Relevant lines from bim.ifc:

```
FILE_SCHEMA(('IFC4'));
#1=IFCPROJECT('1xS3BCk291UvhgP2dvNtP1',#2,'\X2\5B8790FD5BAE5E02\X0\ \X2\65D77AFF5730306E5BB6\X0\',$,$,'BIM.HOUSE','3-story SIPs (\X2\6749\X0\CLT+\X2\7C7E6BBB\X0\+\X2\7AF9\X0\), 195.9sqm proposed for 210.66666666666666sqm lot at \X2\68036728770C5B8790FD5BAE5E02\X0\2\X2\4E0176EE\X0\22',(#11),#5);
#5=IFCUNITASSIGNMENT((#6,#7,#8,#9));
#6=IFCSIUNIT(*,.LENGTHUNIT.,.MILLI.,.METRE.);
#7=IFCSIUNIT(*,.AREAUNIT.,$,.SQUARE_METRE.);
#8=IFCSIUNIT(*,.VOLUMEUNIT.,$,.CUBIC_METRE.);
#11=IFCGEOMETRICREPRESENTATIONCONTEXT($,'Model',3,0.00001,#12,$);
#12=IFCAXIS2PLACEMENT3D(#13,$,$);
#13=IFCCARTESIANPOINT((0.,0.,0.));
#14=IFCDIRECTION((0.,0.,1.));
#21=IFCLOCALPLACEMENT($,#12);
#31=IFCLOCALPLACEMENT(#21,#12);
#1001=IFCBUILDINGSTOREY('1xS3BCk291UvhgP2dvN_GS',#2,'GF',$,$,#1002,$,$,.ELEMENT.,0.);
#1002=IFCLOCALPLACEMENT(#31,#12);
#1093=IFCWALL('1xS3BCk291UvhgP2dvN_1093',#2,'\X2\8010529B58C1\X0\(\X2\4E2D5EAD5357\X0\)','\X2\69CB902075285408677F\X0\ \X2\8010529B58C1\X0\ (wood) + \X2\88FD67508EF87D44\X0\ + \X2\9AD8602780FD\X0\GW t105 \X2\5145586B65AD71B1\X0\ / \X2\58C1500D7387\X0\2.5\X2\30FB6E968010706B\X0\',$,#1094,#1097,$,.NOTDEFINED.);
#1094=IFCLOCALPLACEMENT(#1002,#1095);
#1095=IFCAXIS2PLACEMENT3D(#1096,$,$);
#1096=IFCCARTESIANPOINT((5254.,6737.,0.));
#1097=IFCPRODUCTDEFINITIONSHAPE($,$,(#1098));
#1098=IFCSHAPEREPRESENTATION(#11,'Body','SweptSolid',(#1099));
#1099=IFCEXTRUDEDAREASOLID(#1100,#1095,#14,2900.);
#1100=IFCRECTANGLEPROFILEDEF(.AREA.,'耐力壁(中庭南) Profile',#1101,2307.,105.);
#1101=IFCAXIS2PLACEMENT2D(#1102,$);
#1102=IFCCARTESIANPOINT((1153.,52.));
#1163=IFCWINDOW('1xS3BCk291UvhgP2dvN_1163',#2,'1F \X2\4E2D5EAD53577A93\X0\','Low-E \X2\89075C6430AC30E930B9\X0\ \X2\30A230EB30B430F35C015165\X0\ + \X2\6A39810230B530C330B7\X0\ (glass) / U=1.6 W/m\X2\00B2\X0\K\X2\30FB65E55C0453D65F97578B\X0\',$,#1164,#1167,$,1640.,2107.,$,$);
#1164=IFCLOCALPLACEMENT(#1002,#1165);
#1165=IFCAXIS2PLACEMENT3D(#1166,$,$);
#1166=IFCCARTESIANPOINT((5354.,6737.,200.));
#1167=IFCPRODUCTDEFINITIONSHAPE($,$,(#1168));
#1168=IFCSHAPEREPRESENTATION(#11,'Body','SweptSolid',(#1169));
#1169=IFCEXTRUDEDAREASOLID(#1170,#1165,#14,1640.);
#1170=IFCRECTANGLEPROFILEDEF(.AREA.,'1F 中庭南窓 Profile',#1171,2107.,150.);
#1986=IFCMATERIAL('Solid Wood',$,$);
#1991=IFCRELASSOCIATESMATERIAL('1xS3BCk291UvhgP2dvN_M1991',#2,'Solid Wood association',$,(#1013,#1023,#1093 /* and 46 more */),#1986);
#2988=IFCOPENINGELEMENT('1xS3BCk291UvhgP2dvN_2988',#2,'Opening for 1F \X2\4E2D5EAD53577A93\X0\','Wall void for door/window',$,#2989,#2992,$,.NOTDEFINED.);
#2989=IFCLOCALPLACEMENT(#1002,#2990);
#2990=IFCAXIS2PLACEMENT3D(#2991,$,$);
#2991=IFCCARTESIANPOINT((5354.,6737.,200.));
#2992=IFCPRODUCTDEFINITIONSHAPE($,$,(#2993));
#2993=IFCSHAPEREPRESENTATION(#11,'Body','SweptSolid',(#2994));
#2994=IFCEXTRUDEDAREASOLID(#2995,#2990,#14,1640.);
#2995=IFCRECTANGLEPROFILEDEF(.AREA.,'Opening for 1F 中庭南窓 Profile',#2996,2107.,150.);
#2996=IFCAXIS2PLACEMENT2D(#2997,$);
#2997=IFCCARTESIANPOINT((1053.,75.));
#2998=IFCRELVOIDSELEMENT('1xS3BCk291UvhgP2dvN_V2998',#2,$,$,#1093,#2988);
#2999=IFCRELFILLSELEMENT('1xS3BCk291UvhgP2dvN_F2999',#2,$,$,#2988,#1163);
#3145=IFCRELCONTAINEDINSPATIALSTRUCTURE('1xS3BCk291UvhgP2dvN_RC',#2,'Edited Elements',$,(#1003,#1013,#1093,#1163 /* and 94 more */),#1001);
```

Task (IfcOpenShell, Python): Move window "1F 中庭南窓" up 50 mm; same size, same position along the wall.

```python
import numpy as np
import ifcopenshell
import ifcopenshell.api.geometry
import ifcopenshell.util.placement
import ifcopenshell.util.unit

model = ifcopenshell.open("bim.ifc")
unit_scale = ifcopenshell.util.unit.calculate_unit_scale(model)

window = model.by_guid("1xS3BCk291UvhgP2dvN_1163")
opening = window.FillsVoids[0].RelatingOpeningElement
dz = 50.0

shift = np.array([0.0, 0.0, dz])
# The window is not placed relative to its opening, so move both.
for product in (opening, window):
    matrix = ifcopenshell.util.placement.get_local_placement(product.ObjectPlacement)
    matrix[:3, 3] += shift
    ifcopenshell.api.geometry.edit_object_placement(model, product=product, matrix=matrix, is_si=False)

print(f"moved by {dz * unit_scale:+.3f} m")

model.write("bim_updated.ifc")
```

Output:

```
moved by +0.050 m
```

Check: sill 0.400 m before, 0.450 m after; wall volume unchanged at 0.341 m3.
